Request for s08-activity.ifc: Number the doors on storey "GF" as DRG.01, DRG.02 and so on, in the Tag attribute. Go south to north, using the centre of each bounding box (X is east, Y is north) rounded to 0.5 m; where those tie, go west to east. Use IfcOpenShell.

First a look at what the model holds.

```python
import ifcopenshell
import ifcopenshell.util.element
import ifcopenshell.util.placement

model = ifcopenshell.open("s08-activity.ifc")
print(model.schema)
storey = next(s for s in model.by_type("IfcBuildingStorey") if s.Name == "GF")
doors = [e for e in ifcopenshell.util.element.get_decomposition(storey) if e.is_a("IfcDoor")]
for e in sorted(doors, key=lambda e: e.id()):
    origin = ifcopenshell.util.placement.get_local_placement(e.ObjectPlacement)[:3, 3]
    print(e.id(), e.Tag, e.Name, origin.round(2) + 0.0, sep=" | ")
```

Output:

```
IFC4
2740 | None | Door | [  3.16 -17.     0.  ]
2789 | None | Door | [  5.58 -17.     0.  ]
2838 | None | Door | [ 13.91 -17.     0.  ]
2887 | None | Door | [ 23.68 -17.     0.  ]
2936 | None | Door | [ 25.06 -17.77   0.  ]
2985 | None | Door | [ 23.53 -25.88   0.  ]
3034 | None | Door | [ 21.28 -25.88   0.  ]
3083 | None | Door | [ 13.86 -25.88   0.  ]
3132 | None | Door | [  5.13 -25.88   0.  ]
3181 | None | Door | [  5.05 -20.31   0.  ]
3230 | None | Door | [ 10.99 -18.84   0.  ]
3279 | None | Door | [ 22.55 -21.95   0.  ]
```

```python
import ifcopenshell
import ifcopenshell.geom
import ifcopenshell.util.element
import ifcopenshell.util.shape

model = ifcopenshell.open("s08-activity.ifc")
settings = ifcopenshell.geom.settings()
settings.set("use-world-coords", True)


def centre(element):
    shape = ifcopenshell.geom.create_shape(settings, element)
    return ifcopenshell.util.shape.get_bbox_centroid(shape.geometry)


storey = next(s for s in model.by_type("IfcBuildingStorey") if s.Name == "GF")
doors = [e for e in ifcopenshell.util.element.get_decomposition(storey) if e.is_a("IfcDoor")]

# Insertion points can sit at a corner or the storey origin, so sort by the geometry (in metres).
centres = {e: centre(e) for e in doors}
doors.sort(key=lambda e: (round(centres[e][1] / 0.5), centres[e][0]))

for i, e in enumerate(doors, start=1):
    number = f"DRG.{i:02d}"
    e.Tag = number
    print(e.id(), number)

model.write("s08-activity_v2.ifc")
```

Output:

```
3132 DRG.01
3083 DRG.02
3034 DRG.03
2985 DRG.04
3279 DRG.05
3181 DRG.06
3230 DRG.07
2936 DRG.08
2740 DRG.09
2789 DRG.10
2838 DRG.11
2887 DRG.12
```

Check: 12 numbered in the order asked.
